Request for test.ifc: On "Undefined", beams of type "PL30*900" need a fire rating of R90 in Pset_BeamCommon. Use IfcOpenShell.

First a look at what the model holds.

```python
import ifcopenshell
import ifcopenshell.util.element

model = ifcopenshell.open("test.ifc")
print(model.schema)
storey = next(s for s in model.by_type("IfcBuildingStorey") if s.Name == "Undefined")
beams = [e for e in ifcopenshell.util.element.get_decomposition(storey) if e.is_a("IfcBeam")]
seen = {}
for e in beams:
    element_type = ifcopenshell.util.element.get_type(e)
    key = (element_type.Name if element_type != e and element_type else None, ifcopenshell.util.element.get_pset(e, "Pset_BeamCommon", "FireRating"))
    seen[key] = seen.get(key, 0) + 1
for (name, value), count in sorted(seen.items(), key=str):
    print(count, "x", name, "|", value)
```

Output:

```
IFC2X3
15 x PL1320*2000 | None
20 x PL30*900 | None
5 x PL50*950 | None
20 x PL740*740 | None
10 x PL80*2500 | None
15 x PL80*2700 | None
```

```python
import ifcopenshell
import ifcopenshell.api.pset
import ifcopenshell.util.element

model = ifcopenshell.open("test.ifc")

storey = next(s for s in model.by_type("IfcBuildingStorey") if s.Name == "Undefined")
beams = [e for e in ifcopenshell.util.element.get_decomposition(storey) if e.is_a("IfcBeam")]

count = 0
for e in beams:
    element_type = ifcopenshell.util.element.get_type(e)
    if element_type in (None, e) or element_type.Name != "PL30*900":
        continue
    found = ifcopenshell.util.element.get_pset(e, "Pset_BeamCommon", should_inherit=False)
    if found:
        pset = model.by_id(found["id"])
        if len(ifcopenshell.util.element.get_elements_by_pset(pset)) > 1:
            pset = ifcopenshell.api.pset.unshare_pset(model, products=[e], pset=pset)[0]
    else:
        pset = ifcopenshell.api.pset.add_pset(model, product=e, name="Pset_BeamCommon")
    ifcopenshell.api.pset.edit_pset(model, pset=pset, properties={"FireRating": "R90"})
    count += 1

print(count, "beams updated")

model.write("test_updated.ifc")
```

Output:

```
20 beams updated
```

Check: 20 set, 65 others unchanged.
